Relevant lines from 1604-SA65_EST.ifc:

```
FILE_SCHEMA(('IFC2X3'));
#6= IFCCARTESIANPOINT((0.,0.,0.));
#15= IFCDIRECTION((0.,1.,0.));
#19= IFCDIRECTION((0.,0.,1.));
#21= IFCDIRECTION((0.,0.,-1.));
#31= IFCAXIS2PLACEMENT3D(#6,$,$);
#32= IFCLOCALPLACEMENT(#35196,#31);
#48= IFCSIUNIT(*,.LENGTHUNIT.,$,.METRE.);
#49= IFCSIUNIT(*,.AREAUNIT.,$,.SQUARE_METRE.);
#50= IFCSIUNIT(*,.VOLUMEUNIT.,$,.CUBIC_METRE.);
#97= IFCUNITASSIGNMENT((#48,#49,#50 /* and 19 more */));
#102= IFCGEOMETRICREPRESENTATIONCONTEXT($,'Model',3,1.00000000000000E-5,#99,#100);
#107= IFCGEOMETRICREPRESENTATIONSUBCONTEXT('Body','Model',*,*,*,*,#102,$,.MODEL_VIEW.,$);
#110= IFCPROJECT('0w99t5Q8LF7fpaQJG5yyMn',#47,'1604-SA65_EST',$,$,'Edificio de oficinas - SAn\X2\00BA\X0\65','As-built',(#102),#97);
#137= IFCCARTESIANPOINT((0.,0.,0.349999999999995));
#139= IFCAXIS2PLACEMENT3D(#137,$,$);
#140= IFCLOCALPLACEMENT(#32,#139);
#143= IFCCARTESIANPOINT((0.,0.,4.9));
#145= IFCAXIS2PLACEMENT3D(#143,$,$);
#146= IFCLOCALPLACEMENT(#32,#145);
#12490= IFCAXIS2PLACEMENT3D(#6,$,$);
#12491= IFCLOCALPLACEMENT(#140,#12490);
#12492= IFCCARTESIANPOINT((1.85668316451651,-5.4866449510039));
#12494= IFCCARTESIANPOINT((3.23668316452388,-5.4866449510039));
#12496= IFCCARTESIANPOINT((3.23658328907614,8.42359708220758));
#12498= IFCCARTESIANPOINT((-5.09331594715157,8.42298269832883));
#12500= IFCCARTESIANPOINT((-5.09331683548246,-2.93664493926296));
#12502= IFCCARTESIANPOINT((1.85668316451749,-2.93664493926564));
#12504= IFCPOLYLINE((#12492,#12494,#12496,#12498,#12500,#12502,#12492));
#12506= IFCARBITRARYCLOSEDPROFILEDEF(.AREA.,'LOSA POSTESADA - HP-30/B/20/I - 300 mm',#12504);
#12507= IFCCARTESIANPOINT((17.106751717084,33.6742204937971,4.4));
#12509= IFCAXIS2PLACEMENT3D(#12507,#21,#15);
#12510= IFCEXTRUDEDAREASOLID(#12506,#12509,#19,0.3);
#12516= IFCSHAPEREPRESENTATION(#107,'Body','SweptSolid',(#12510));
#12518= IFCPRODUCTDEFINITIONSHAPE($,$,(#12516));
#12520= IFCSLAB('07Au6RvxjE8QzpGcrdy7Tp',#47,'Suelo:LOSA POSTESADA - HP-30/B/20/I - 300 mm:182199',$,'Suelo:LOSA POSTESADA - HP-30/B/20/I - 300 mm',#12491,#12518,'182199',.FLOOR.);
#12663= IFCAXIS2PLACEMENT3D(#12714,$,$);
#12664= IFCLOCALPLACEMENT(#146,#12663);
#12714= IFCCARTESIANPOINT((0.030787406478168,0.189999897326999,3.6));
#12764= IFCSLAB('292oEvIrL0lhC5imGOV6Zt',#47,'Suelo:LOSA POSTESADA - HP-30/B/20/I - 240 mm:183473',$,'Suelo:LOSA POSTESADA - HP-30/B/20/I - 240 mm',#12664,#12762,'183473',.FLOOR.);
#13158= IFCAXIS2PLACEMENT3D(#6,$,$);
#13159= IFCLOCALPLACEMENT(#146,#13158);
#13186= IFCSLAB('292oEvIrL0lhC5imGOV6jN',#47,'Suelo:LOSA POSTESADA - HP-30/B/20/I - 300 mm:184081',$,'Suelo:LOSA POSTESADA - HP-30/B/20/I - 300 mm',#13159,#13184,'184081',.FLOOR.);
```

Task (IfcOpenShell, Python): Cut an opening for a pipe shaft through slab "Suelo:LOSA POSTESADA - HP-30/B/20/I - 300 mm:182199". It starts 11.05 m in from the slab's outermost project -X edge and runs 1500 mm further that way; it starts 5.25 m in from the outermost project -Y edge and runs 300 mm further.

```python
import numpy as np
import ifcopenshell
import ifcopenshell.api.feature
import ifcopenshell.api.geometry
import ifcopenshell.api.root
import ifcopenshell.geom
import ifcopenshell.util.placement
import ifcopenshell.util.representation
import ifcopenshell.util.shape
import ifcopenshell.util.unit

model = ifcopenshell.open("1604-SA65_EST.ifc")
unit_scale = ifcopenshell.util.unit.calculate_unit_scale(model)
settings = ifcopenshell.geom.settings()


def volume(element):
    """Net volume in cubic metres, openings subtracted."""
    shape = ifcopenshell.geom.create_shape(settings, element)
    return ifcopenshell.util.shape.get_volume(shape.geometry)


slab = model.by_id(12520)
before = volume(slab)

# Extent in the slab's own axes, in metres. The edges named are its -X and -Y sides.
slab_shape = ifcopenshell.geom.create_shape(settings, slab)
vertices = ifcopenshell.util.shape.get_vertices(slab_shape.geometry)
x_min, y_min, bottom = vertices.min(axis=0)
top = vertices[:, 2].max()

opening = ifcopenshell.api.root.create_entity(model, ifc_class="IfcOpeningElement", name="Pipe shaft opening")
context = ifcopenshell.util.representation.get_context(model, "Model", "Body", "MODEL_VIEW")
width, depth = 1.5, 0.3
outline = [(0.0, 0.0), (width, 0.0), (width, depth), (0.0, depth), (0.0, 0.0)]
# Overshoot both faces by 50 mm so the cut is clean.
shape = ifcopenshell.api.geometry.add_slab_representation(
    model, context=context, depth=top - bottom + 0.1, polyline=outline
)
ifcopenshell.api.geometry.assign_representation(model, product=opening, representation=shape)

matrix = ifcopenshell.util.placement.get_local_placement(slab.ObjectPlacement)
matrix[:, 3] = matrix @ np.append(np.array([x_min + 11.05, y_min + 5.25, bottom - 0.05]) / unit_scale, 1.0)
ifcopenshell.api.geometry.edit_object_placement(model, product=opening, matrix=matrix, is_si=False)
ifcopenshell.api.feature.add_feature(model, feature=opening, element=slab)

after = volume(slab)

print(f"slab volume {before:.3f} -> {after:.3f} m3")

model.write("1604-SA65_EST-out.ifc")
```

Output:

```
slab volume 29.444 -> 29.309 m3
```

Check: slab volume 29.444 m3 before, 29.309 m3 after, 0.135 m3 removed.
